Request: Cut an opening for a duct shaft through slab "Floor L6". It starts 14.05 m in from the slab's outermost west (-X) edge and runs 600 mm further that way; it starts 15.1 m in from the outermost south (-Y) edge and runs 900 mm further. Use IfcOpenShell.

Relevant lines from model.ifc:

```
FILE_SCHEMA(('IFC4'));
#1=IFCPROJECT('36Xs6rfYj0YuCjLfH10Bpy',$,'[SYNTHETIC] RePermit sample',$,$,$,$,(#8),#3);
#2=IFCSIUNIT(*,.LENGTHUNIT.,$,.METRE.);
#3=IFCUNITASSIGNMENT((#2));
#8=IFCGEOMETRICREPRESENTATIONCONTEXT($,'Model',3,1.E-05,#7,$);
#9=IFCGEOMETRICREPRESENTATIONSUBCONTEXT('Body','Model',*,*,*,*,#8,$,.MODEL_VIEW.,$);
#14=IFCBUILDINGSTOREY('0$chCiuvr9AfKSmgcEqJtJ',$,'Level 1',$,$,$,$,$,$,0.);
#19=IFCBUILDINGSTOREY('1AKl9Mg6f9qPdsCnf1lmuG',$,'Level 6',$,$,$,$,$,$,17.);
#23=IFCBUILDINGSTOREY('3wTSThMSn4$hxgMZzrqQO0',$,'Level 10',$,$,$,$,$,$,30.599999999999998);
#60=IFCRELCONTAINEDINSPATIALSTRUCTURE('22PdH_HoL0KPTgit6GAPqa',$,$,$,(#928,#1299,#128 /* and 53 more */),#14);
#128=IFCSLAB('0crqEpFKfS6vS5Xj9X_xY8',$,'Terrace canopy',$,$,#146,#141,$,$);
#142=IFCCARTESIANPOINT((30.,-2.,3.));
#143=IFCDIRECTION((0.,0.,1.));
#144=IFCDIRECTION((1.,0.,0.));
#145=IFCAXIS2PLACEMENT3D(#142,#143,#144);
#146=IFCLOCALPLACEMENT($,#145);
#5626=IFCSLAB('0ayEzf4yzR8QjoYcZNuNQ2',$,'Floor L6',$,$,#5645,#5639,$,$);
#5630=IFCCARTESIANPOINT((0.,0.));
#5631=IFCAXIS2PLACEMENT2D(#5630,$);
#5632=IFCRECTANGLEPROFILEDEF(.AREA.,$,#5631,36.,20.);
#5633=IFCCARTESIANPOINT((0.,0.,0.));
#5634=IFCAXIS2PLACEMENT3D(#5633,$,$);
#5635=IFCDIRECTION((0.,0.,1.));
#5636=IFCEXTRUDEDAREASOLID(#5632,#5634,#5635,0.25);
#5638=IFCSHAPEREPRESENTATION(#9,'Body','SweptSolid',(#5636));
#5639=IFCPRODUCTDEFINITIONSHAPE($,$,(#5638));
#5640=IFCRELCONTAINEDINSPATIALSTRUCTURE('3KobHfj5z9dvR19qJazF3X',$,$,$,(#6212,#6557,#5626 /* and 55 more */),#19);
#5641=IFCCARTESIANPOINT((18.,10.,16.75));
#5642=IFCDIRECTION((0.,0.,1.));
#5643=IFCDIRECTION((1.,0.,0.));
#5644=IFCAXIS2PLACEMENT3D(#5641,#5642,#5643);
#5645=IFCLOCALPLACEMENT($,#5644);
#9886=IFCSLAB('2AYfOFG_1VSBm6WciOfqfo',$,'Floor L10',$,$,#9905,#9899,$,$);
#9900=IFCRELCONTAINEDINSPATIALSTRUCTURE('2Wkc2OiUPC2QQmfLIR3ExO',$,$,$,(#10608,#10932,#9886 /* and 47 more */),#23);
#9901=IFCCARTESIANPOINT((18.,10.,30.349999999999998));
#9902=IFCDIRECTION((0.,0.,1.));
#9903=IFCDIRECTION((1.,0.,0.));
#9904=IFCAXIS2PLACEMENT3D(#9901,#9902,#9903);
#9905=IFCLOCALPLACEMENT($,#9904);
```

```python
import numpy as np
import ifcopenshell
import ifcopenshell.api.feature
import ifcopenshell.api.geometry
import ifcopenshell.api.root
import ifcopenshell.geom
import ifcopenshell.util.placement
import ifcopenshell.util.representation
import ifcopenshell.util.shape
import ifcopenshell.util.unit

model = ifcopenshell.open("model.ifc")
unit_scale = ifcopenshell.util.unit.calculate_unit_scale(model)
settings = ifcopenshell.geom.settings()


def volume(element):
    """Net volume in cubic metres, openings subtracted."""
    shape = ifcopenshell.geom.create_shape(settings, element)
    return ifcopenshell.util.shape.get_volume(shape.geometry)


slab = model.by_id(5626)
before = volume(slab)

# Extent in the slab's own axes, in metres. The edges named are its -X and -Y sides.
slab_shape = ifcopenshell.geom.create_shape(settings, slab)
vertices = ifcopenshell.util.shape.get_vertices(slab_shape.geometry)
x_min, y_min, bottom = vertices.min(axis=0)
top = vertices[:, 2].max()

opening = ifcopenshell.api.root.create_entity(model, ifc_class="IfcOpeningElement", name="Duct shaft opening", predefined_type="OPENING")
context = ifcopenshell.util.representation.get_context(model, "Model", "Body", "MODEL_VIEW")
width, depth = 0.6, 0.9
outline = [(0.0, 0.0), (width, 0.0), (width, depth), (0.0, depth), (0.0, 0.0)]
# Overshoot both faces by 50 mm so the cut is clean.
shape = ifcopenshell.api.geometry.add_slab_representation(
    model, context=context, depth=top - bottom + 0.1, polyline=outline
)
ifcopenshell.api.geometry.assign_representation(model, product=opening, representation=shape)

matrix = ifcopenshell.util.placement.get_local_placement(slab.ObjectPlacement)
matrix[:, 3] = matrix @ np.append(np.array([x_min + 14.05, y_min + 15.1, bottom - 0.05]) / unit_scale, 1.0)
ifcopenshell.api.geometry.edit_object_placement(model, product=opening, matrix=matrix, is_si=False)
ifcopenshell.api.feature.add_feature(model, feature=opening, element=slab)

after = volume(slab)

print(f"slab volume {before:.3f} -> {after:.3f} m3")

model.write("model-out.ifc")
```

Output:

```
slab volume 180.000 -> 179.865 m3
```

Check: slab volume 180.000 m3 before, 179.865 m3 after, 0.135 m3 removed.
